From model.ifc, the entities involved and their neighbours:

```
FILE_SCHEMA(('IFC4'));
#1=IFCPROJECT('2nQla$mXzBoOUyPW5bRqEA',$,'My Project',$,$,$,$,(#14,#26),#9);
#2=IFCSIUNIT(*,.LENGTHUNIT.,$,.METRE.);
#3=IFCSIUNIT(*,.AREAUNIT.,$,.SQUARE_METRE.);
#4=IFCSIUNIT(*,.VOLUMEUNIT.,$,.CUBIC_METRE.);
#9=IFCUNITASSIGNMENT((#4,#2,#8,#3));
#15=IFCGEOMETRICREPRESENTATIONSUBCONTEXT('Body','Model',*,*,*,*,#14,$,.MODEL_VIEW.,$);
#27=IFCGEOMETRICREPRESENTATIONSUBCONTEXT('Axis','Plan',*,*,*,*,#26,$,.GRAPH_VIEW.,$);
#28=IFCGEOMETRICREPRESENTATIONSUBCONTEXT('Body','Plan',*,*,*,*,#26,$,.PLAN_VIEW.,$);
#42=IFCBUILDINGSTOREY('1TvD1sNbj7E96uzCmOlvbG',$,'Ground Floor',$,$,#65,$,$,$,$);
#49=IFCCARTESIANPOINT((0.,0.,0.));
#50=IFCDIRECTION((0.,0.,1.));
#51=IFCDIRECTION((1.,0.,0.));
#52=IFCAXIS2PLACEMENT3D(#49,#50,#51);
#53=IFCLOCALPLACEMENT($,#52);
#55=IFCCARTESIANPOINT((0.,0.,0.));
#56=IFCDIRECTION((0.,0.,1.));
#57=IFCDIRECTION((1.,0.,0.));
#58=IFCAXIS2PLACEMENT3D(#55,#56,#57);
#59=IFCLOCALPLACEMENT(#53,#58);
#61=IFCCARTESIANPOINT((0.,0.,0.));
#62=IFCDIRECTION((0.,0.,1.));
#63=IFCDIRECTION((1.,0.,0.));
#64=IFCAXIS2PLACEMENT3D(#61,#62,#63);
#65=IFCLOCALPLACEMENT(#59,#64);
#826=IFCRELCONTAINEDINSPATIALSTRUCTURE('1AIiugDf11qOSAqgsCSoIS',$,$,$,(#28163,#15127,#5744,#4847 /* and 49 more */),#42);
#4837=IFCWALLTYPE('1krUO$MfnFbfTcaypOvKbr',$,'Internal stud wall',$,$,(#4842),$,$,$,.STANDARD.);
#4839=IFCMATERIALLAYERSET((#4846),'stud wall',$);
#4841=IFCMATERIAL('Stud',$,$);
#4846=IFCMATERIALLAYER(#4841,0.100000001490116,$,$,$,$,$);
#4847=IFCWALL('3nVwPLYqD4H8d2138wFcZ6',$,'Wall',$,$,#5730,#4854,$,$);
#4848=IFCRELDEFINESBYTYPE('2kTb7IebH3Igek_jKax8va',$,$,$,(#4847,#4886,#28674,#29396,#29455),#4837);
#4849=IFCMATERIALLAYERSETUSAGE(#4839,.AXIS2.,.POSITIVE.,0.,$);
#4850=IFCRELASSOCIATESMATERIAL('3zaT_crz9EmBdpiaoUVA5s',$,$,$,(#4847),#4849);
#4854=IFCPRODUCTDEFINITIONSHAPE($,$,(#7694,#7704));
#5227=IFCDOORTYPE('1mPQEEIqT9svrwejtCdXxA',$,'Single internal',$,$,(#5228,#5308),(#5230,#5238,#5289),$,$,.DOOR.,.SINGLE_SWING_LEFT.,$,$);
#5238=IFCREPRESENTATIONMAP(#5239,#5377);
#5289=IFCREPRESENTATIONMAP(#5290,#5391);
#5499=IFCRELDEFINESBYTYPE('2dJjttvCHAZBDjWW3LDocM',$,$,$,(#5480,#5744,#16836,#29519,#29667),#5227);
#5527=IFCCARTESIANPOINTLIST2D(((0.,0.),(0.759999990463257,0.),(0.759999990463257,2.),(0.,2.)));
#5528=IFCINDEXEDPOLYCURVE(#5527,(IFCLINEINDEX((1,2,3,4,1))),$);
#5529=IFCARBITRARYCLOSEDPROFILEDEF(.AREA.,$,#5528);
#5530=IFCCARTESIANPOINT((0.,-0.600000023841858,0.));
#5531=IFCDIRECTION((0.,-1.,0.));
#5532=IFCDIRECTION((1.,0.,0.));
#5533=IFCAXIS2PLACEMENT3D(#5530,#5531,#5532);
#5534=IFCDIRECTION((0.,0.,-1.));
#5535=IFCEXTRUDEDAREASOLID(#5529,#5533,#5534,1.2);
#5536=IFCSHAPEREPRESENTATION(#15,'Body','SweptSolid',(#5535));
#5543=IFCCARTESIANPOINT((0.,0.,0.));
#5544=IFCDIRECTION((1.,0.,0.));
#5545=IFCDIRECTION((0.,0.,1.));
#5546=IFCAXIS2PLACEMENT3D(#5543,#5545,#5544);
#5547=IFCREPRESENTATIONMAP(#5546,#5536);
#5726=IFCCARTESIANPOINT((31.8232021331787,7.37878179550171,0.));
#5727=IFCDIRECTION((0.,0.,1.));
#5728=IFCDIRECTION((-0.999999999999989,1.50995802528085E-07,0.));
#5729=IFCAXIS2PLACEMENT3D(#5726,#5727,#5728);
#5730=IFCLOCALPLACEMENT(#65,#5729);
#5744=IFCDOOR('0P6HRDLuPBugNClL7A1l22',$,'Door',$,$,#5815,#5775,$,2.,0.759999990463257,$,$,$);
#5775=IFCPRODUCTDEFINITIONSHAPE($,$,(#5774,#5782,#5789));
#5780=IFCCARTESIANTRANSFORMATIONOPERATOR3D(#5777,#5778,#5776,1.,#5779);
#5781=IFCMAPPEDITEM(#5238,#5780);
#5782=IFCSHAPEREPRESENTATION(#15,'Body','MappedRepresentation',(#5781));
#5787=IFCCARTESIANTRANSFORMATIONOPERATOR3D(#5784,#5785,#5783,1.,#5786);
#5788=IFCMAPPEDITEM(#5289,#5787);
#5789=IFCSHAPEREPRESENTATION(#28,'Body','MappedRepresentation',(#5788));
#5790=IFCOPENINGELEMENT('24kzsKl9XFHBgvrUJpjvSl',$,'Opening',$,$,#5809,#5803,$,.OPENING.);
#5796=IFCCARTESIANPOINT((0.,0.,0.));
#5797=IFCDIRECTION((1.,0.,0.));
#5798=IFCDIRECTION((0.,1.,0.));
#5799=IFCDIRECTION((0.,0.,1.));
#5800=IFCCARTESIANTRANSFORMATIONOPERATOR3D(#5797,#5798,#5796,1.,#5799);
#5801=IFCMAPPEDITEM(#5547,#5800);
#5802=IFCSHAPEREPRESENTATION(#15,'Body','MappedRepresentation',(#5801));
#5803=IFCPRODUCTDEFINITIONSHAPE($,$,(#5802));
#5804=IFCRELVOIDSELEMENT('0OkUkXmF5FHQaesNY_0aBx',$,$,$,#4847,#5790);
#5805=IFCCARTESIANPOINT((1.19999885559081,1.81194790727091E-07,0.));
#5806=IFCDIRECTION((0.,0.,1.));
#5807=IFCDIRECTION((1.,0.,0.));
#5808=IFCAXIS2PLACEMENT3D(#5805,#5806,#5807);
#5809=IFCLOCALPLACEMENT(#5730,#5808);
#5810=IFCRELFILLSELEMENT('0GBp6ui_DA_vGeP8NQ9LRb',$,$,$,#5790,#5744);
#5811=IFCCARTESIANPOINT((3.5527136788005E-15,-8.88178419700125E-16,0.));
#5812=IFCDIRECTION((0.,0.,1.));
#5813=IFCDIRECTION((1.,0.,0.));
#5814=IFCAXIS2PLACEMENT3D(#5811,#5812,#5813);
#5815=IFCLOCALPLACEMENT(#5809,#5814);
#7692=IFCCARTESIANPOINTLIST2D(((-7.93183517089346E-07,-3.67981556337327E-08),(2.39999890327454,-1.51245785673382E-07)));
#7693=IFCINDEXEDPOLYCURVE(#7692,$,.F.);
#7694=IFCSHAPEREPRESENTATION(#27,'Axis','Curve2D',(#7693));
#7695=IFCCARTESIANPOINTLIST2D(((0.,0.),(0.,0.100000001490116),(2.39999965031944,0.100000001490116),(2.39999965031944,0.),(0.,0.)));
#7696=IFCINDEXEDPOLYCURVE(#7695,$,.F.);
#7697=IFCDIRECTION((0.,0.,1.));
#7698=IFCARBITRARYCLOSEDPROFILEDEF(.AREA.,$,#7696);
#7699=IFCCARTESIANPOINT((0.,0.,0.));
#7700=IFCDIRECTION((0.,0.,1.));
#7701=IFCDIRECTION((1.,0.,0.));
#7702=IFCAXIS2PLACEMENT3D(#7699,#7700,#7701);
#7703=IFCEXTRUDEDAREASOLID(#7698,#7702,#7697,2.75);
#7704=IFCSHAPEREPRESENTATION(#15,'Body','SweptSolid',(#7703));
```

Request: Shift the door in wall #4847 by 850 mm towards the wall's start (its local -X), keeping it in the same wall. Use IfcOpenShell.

```python
import ifcopenshell
import ifcopenshell.api.geometry
import ifcopenshell.util.placement
import ifcopenshell.util.unit

model = ifcopenshell.open("model.ifc")
unit_scale = ifcopenshell.util.unit.calculate_unit_scale(model)

door = model.by_guid("0P6HRDLuPBugNClL7A1l22")
opening = door.FillsVoids[0].RelatingOpeningElement
wall = opening.VoidsElements[0].RelatingBuildingElement

wall_matrix = ifcopenshell.util.placement.get_local_placement(wall.ObjectPlacement)
shift = wall_matrix[:3, 0] * -0.85 / unit_scale
before = ifcopenshell.util.placement.get_local_placement(door.ObjectPlacement)[:3, 3].copy()

# The door is placed relative to its opening, so it follows when the opening moves.
matrix = ifcopenshell.util.placement.get_local_placement(opening.ObjectPlacement)
matrix[:3, 3] += shift
ifcopenshell.api.geometry.edit_object_placement(
    model, product=opening, matrix=matrix, is_si=False, should_transform_children=True
)

after = ifcopenshell.util.placement.get_local_placement(door.ObjectPlacement)[:3, 3]
print("door moved by", (after - before).round(3) + 0.0)

model.write("model_updated.ifc")
```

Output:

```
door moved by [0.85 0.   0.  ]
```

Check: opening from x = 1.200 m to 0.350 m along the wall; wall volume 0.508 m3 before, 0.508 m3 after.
